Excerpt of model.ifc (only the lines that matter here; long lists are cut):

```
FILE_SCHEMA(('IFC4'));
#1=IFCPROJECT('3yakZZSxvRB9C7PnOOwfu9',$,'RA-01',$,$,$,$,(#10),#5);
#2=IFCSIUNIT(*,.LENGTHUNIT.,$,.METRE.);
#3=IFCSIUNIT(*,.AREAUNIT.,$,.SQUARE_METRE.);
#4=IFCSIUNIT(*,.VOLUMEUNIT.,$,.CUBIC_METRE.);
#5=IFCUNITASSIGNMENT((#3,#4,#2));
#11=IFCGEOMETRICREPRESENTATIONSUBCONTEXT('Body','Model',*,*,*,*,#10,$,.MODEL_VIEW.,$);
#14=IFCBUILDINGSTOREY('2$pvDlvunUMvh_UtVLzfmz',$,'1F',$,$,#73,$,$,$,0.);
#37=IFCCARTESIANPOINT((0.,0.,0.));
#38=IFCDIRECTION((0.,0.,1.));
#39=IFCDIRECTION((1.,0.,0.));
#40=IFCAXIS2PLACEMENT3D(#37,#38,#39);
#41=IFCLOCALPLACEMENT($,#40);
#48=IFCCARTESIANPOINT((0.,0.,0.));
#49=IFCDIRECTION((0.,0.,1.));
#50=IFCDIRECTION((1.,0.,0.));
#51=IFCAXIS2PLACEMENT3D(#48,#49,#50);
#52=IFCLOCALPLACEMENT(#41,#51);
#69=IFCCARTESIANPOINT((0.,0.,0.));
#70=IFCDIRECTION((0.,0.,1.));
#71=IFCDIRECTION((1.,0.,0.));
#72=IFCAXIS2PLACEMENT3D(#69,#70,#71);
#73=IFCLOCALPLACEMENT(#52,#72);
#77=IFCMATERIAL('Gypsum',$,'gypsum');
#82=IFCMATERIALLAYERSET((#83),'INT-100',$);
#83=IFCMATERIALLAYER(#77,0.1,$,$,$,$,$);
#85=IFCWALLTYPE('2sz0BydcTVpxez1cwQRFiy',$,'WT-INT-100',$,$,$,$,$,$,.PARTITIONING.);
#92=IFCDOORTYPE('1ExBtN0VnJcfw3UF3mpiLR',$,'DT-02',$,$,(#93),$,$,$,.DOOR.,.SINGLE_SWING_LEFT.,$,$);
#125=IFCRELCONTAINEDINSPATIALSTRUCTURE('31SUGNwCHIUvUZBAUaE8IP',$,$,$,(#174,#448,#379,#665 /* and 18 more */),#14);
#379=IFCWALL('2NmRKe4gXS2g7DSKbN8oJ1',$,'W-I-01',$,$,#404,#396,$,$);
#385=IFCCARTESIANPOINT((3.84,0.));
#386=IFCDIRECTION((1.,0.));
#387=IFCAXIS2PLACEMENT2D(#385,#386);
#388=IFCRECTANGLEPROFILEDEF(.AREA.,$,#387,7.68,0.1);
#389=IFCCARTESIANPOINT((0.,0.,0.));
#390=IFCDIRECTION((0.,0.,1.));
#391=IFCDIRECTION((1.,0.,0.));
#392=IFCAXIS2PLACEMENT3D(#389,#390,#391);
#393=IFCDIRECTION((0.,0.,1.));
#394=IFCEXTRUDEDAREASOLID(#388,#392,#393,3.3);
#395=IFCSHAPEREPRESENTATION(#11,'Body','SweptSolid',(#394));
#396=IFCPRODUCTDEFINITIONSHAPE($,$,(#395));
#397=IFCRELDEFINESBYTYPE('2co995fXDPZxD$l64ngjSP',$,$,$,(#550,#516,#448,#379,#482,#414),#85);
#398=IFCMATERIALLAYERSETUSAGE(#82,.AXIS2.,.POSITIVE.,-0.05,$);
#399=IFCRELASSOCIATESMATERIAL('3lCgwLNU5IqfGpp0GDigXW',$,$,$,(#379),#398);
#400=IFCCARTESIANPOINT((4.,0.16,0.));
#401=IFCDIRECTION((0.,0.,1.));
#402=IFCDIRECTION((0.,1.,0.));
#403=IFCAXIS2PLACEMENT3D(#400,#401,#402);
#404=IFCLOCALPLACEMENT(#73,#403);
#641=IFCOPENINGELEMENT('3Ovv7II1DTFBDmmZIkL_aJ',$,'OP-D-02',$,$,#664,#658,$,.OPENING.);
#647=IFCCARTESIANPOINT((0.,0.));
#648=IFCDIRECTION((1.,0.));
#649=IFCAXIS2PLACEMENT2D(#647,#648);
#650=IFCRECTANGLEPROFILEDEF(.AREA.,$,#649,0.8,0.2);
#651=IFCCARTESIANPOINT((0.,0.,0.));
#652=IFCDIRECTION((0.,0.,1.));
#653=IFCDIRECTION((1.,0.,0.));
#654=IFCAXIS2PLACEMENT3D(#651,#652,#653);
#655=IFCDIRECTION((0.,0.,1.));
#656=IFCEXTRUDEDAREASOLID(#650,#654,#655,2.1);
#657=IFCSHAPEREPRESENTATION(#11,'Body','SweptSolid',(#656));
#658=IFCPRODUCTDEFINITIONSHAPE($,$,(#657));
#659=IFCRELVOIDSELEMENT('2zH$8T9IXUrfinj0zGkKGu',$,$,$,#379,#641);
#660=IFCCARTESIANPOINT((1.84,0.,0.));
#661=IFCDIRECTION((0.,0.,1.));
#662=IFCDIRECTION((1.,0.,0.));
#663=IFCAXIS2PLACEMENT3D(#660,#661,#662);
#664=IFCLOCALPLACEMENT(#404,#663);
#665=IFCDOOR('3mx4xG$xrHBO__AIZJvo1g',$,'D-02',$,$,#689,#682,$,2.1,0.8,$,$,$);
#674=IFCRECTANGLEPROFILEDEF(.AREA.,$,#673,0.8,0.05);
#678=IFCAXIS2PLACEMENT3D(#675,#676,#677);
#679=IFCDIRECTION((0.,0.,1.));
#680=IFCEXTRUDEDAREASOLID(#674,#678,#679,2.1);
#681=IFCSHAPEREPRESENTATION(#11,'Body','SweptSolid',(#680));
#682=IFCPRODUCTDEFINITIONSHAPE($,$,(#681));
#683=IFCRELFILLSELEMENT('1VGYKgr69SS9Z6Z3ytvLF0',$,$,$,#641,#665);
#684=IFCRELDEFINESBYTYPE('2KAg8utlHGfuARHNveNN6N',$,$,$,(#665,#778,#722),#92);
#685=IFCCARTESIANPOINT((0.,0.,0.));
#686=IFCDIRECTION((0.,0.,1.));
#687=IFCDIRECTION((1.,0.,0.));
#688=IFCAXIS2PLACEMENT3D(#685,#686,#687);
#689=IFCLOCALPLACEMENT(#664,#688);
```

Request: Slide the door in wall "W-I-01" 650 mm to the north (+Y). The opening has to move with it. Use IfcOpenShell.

```python
import ifcopenshell
import ifcopenshell.api.geometry
import ifcopenshell.util.placement

model = ifcopenshell.open("model.ifc")

door = model.by_id(665)
opening = door.FillsVoids[0].RelatingOpeningElement
wall = opening.VoidsElements[0].RelatingBuildingElement

wall_matrix = ifcopenshell.util.placement.get_local_placement(wall.ObjectPlacement)
shift = wall_matrix[:3, 0] * 0.65
before = ifcopenshell.util.placement.get_local_placement(door.ObjectPlacement)[:3, 3].copy()

# The door is placed relative to its opening, so it follows when the opening moves.
matrix = ifcopenshell.util.placement.get_local_placement(opening.ObjectPlacement)
matrix[:3, 3] += shift
ifcopenshell.api.geometry.edit_object_placement(
    model, product=opening, matrix=matrix, is_si=False, should_transform_children=True
)

after = ifcopenshell.util.placement.get_local_placement(door.ObjectPlacement)[:3, 3]
print("door moved by", (after - before).round(3) + 0.0)

model.write("model_updated.ifc")
```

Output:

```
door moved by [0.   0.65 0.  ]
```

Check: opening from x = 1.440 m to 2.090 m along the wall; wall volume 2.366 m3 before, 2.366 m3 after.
